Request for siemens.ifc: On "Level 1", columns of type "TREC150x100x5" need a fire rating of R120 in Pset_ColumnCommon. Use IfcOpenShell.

First a look at what the model holds.

```python
import ifcopenshell
import ifcopenshell.util.element

model = ifcopenshell.open("siemens.ifc")
print(model.schema)
storey = next(s for s in model.by_type("IfcBuildingStorey") if s.Name == "Level 1")
columns = [e for e in ifcopenshell.util.element.get_decomposition(storey) if e.is_a("IfcColumn")]
seen = {}
for e in columns:
    element_type = ifcopenshell.util.element.get_type(e)
    key = (element_type.Name if element_type != e and element_type else None, ifcopenshell.util.element.get_pset(e, "Pset_ColumnCommon", "FireRating"))
    seen[key] = seen.get(key, 0) + 1
for (name, value), count in sorted(seen.items(), key=str):
    print(count, "x", name, "|", value)
```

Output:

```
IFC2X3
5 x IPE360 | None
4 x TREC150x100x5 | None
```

```python
import ifcopenshell
import ifcopenshell.api.pset
import ifcopenshell.util.element

model = ifcopenshell.open("siemens.ifc")

storey = next(s for s in model.by_type("IfcBuildingStorey") if s.Name == "Level 1")
columns = [e for e in ifcopenshell.util.element.get_decomposition(storey) if e.is_a("IfcColumn")]

count = 0
for e in columns:
    element_type = ifcopenshell.util.element.get_type(e)
    if element_type in (None, e) or element_type.Name != "TREC150x100x5":
        continue
    # add_pset returns the element's existing set when there is one.
    pset = ifcopenshell.api.pset.add_pset(model, product=e, name="Pset_ColumnCommon")
    ifcopenshell.api.pset.edit_pset(model, pset=pset, properties={"FireRating": "R120"})
    count += 1

print(count, "columns updated")

model.write("siemens_edited.ifc")
```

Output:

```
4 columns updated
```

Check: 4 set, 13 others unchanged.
